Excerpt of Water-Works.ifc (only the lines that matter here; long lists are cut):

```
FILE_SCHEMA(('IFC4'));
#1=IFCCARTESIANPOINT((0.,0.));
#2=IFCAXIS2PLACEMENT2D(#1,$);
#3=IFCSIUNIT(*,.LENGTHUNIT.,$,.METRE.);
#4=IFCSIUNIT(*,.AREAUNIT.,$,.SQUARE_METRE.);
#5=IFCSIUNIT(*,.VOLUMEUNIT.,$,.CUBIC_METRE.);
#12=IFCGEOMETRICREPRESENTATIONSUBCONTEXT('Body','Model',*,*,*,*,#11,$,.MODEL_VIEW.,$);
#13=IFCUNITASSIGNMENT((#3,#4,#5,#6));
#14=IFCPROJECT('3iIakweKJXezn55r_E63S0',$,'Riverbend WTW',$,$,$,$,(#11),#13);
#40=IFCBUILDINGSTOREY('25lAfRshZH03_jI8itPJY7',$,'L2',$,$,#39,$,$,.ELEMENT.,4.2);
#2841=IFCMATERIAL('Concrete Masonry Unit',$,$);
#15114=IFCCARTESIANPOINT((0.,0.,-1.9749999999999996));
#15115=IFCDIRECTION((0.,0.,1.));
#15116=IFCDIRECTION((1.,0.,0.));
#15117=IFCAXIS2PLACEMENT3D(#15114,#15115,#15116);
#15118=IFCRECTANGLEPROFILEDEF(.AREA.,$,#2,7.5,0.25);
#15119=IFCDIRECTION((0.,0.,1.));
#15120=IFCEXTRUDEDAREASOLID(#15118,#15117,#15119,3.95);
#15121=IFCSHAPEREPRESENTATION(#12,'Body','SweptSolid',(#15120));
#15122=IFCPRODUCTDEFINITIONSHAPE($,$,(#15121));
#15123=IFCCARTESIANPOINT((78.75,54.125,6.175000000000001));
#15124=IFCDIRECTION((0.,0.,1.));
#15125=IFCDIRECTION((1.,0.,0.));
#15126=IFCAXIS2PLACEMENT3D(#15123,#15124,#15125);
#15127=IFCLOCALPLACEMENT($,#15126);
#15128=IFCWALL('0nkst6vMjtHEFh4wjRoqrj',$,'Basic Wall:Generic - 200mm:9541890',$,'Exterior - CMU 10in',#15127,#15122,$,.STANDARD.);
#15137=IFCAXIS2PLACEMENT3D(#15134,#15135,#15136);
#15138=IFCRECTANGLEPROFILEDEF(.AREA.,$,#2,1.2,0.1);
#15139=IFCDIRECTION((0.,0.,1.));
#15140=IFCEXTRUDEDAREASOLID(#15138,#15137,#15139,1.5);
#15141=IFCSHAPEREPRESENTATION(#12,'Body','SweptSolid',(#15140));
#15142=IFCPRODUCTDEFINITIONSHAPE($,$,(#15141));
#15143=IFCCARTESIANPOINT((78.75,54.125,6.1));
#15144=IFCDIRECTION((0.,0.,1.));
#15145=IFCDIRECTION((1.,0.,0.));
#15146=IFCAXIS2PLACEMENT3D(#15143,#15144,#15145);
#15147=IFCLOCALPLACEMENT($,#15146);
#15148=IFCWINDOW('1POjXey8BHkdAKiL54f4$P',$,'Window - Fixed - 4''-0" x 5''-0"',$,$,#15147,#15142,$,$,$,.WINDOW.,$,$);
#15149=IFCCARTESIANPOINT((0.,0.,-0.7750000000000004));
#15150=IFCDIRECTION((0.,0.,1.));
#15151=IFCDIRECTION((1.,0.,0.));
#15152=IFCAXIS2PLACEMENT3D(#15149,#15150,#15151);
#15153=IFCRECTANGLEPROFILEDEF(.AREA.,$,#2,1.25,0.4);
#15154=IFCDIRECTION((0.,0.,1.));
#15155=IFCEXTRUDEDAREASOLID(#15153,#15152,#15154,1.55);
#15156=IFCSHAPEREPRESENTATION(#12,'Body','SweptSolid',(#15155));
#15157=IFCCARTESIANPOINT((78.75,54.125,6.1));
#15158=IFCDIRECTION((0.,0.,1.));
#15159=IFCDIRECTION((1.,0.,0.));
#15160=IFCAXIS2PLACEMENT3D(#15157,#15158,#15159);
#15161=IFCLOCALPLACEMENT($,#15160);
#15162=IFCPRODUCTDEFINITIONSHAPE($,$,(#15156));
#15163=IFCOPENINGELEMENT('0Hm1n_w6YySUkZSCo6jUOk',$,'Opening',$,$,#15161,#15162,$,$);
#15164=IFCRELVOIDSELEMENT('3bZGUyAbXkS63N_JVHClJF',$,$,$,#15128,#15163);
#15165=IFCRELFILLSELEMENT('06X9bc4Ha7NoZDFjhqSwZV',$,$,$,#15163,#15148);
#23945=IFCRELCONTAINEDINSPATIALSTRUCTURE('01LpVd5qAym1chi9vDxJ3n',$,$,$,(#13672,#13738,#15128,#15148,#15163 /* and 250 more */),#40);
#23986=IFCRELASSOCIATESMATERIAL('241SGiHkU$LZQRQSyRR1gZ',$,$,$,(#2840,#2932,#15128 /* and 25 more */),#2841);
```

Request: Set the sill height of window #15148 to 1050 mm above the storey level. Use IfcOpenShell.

```python
import numpy as np
import ifcopenshell
import ifcopenshell.api.geometry
import ifcopenshell.geom
import ifcopenshell.util.element
import ifcopenshell.util.placement
import ifcopenshell.util.shape
import ifcopenshell.util.unit

model = ifcopenshell.open("Water-Works.ifc")
unit_scale = ifcopenshell.util.unit.calculate_unit_scale(model)

window = model.by_guid("1POjXey8BHkdAKiL54f4$P")
opening = window.FillsVoids[0].RelatingOpeningElement
storey = ifcopenshell.util.element.get_container(window, ifc_class="IfcBuildingStorey")
level = ifcopenshell.util.placement.get_local_placement(storey.ObjectPlacement)[2, 3]

# The opening's origin need not be at the sill, so measure its lowest point.
shape = ifcopenshell.geom.create_shape(ifcopenshell.geom.settings(), opening)
bottom = ifcopenshell.util.shape.get_shape_bottom_elevation(shape, shape.geometry) / unit_scale
dz = level + 1.05 / unit_scale - bottom

shift = np.array([0.0, 0.0, dz])
# The window is not placed relative to its opening, so move both.
for product in (opening, window):
    matrix = ifcopenshell.util.placement.get_local_placement(product.ObjectPlacement)
    matrix[:3, 3] += shift
    ifcopenshell.api.geometry.edit_object_placement(model, product=product, matrix=matrix, is_si=False)

print(f"moved by {dz * unit_scale:+.3f} m")

model.write("Water-Works-out.ifc")
```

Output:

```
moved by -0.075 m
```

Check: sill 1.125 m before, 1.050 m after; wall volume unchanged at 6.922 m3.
